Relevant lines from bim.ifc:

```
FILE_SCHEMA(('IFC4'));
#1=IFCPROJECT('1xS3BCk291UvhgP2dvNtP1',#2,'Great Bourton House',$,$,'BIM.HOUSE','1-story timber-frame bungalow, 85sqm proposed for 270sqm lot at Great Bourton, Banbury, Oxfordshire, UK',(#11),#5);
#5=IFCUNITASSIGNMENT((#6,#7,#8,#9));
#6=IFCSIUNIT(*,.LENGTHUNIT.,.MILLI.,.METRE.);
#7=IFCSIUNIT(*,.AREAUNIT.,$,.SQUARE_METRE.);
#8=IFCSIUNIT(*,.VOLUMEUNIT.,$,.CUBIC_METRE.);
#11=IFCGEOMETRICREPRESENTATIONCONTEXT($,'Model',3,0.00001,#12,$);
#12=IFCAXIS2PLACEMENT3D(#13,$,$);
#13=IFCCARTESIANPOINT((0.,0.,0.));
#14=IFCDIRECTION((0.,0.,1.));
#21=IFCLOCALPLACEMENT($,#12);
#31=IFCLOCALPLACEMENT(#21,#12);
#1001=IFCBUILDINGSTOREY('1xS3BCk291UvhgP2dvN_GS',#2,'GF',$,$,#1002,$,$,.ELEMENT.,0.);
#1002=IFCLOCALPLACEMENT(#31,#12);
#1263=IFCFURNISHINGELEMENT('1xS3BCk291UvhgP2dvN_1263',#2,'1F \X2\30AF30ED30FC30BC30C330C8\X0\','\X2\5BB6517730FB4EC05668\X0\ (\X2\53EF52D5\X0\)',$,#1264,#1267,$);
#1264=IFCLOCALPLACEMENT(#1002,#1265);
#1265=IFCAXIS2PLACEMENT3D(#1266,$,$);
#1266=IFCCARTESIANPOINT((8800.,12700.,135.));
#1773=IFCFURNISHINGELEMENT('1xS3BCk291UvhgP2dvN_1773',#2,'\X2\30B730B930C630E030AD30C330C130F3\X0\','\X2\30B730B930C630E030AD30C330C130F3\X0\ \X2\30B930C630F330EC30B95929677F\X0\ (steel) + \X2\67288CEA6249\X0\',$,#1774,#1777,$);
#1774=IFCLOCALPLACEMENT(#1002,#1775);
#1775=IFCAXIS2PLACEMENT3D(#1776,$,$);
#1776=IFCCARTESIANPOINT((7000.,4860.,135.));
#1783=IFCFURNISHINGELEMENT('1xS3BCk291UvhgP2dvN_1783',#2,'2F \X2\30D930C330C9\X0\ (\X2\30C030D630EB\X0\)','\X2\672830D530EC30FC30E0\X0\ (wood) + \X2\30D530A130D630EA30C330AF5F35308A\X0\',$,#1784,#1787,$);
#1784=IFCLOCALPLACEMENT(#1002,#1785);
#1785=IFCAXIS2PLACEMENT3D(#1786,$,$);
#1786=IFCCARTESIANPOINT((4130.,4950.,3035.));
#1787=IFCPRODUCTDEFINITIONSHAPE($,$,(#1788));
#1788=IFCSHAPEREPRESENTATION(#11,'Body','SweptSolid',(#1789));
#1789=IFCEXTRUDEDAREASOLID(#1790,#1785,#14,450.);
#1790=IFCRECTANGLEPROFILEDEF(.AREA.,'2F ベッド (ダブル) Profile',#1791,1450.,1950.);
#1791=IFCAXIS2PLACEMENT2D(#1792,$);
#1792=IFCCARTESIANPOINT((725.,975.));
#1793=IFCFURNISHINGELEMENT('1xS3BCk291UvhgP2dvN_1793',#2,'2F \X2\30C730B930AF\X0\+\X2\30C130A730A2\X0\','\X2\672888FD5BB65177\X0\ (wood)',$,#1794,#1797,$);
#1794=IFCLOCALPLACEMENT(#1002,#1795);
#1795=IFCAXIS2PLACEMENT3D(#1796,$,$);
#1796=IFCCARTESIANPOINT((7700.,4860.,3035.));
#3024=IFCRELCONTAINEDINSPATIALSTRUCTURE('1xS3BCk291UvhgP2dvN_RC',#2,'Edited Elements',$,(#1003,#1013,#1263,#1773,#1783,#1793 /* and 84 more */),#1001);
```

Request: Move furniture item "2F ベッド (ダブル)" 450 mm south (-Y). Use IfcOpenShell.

```python
import ifcopenshell
import ifcopenshell.api.geometry
import ifcopenshell.util.placement

model = ifcopenshell.open("bim.ifc")

item = model.by_guid("1xS3BCk291UvhgP2dvN_1783")
matrix = ifcopenshell.util.placement.get_local_placement(item.ObjectPlacement)
matrix[1, 3] -= 450.0
ifcopenshell.api.geometry.edit_object_placement(model, product=item, matrix=matrix, is_si=False)

print(ifcopenshell.util.placement.get_local_placement(item.ObjectPlacement).round(3) + 0.0)

model.write("bim_rev.ifc")
```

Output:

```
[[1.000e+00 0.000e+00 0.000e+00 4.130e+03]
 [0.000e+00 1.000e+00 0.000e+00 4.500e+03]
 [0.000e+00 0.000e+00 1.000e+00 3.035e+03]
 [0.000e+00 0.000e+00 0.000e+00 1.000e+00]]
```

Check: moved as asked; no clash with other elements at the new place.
